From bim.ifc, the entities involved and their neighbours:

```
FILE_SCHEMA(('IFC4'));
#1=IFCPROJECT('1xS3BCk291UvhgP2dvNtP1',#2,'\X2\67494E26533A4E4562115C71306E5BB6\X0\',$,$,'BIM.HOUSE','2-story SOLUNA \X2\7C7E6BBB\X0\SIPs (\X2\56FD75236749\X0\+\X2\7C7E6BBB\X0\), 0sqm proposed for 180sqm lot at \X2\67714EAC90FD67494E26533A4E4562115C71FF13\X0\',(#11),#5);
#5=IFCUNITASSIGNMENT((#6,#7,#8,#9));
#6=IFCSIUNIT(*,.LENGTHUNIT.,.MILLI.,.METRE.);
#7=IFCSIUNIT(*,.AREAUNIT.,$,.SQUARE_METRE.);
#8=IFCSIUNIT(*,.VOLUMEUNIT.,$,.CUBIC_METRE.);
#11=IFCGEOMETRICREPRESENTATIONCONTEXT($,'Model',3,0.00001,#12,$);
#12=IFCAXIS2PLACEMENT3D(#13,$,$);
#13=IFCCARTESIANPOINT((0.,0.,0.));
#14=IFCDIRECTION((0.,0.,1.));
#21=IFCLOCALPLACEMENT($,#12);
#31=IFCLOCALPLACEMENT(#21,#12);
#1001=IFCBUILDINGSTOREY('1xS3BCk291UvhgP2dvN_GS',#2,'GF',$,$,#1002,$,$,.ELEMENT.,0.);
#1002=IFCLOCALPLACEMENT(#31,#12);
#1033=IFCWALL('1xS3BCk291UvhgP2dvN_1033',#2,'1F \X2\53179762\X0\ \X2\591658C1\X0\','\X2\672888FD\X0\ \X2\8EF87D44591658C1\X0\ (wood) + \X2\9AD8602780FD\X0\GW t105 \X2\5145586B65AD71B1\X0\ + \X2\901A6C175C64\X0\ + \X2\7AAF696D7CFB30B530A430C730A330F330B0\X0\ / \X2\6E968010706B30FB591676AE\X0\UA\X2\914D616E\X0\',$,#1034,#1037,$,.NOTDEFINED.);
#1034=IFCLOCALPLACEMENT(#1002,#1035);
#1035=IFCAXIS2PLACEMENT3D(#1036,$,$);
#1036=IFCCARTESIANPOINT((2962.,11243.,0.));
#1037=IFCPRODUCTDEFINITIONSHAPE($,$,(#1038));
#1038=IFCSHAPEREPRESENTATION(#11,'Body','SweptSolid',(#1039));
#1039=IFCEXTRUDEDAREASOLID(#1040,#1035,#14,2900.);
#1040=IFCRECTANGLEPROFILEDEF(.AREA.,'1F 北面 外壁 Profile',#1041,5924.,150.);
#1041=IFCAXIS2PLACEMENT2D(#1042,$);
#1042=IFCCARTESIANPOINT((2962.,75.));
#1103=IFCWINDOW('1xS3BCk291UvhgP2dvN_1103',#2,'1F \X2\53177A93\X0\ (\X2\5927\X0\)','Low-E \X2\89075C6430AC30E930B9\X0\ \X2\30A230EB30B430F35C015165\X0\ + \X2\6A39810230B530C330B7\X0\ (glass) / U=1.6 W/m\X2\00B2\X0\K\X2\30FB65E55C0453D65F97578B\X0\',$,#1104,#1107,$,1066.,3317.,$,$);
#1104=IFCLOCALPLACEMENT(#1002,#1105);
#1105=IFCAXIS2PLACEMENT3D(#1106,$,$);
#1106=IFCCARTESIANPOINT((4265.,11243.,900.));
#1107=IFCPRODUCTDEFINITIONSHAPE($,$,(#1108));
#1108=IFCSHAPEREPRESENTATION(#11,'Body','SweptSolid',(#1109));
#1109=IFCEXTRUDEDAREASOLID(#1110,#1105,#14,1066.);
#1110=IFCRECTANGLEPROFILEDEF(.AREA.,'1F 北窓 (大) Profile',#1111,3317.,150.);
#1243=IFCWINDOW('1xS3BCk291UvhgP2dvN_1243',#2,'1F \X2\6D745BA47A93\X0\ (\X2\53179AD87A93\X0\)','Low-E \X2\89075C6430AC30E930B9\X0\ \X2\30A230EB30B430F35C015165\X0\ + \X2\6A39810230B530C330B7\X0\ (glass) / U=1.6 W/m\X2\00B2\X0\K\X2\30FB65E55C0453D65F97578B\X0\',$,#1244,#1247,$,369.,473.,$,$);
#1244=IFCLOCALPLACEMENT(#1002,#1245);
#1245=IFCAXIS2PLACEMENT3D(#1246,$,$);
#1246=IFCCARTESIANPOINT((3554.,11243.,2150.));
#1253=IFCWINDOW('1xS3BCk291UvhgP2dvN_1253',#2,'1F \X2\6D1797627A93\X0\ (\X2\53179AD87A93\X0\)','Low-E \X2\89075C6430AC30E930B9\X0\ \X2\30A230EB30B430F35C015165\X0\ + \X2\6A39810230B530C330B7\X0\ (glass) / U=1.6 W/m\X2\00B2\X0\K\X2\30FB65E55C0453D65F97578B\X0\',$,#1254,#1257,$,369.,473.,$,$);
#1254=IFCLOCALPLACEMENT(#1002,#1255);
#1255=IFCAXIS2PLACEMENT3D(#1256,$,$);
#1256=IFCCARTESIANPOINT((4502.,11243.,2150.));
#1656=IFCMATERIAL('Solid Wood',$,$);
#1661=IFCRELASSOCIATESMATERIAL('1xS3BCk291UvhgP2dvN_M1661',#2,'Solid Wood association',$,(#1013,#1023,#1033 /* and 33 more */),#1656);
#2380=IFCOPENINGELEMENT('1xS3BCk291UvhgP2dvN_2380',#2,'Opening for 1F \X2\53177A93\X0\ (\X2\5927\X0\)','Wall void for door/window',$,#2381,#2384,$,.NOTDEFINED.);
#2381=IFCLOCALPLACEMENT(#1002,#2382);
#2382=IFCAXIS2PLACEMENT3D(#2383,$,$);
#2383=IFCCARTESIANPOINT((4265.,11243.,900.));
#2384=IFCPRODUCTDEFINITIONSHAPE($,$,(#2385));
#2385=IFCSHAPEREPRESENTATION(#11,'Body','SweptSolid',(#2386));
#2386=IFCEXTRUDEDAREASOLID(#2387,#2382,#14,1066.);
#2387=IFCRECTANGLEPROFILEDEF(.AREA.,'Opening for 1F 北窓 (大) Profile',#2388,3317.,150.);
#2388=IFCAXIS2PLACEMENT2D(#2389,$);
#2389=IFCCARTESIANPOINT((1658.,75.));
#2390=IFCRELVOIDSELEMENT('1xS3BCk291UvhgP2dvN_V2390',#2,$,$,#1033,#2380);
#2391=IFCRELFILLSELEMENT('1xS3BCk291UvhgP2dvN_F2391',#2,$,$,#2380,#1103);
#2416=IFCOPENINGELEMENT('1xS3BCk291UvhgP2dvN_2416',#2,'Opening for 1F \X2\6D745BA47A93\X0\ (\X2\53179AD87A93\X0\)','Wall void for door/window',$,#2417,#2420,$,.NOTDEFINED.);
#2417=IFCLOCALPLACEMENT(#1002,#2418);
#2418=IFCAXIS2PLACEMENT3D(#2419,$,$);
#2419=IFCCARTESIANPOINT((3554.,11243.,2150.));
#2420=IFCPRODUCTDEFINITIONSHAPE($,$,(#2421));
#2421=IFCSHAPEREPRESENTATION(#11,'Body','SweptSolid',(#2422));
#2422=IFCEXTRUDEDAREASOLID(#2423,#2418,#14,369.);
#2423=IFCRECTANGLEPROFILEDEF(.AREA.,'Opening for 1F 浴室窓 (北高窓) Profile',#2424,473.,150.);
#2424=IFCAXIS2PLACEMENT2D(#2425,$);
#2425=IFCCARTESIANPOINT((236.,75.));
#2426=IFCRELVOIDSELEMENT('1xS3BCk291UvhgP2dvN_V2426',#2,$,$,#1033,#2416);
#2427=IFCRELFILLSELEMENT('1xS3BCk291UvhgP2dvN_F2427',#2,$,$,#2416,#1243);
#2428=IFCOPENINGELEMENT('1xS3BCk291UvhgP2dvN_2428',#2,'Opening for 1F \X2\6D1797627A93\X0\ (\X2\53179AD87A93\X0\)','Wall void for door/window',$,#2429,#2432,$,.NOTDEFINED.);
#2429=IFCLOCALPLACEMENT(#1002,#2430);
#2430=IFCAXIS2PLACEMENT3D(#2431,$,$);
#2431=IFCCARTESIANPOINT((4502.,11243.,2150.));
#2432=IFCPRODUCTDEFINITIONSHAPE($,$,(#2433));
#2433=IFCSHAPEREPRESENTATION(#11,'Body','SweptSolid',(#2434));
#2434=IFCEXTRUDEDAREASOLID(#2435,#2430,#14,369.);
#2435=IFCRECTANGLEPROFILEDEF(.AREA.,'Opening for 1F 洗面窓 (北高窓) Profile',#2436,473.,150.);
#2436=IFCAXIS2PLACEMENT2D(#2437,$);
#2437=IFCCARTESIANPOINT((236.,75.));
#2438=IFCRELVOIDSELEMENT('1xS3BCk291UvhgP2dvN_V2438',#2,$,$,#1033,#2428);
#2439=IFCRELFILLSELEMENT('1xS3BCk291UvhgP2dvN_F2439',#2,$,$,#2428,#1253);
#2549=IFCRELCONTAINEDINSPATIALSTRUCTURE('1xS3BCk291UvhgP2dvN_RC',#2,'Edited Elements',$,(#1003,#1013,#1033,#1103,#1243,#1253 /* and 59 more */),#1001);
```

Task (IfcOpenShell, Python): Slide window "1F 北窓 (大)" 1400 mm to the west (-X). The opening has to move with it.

```python
import ifcopenshell
import ifcopenshell.api.geometry
import ifcopenshell.util.placement
import ifcopenshell.util.unit

model = ifcopenshell.open("bim.ifc")
unit_scale = ifcopenshell.util.unit.calculate_unit_scale(model)

window = model.by_guid("1xS3BCk291UvhgP2dvN_1103")
opening = window.FillsVoids[0].RelatingOpeningElement
wall = opening.VoidsElements[0].RelatingBuildingElement

wall_matrix = ifcopenshell.util.placement.get_local_placement(wall.ObjectPlacement)
shift = wall_matrix[:3, 0] * -1.4 / unit_scale
before = ifcopenshell.util.placement.get_local_placement(window.ObjectPlacement)[:3, 3].copy()

# The window is not placed relative to its opening, so move both.
for product in (opening, window):
    matrix = ifcopenshell.util.placement.get_local_placement(product.ObjectPlacement)
    matrix[:3, 3] += shift
    ifcopenshell.api.geometry.edit_object_placement(model, product=product, matrix=matrix, is_si=False)

after = ifcopenshell.util.placement.get_local_placement(window.ObjectPlacement)[:3, 3]
print("window moved by", (after - before).round(3) + 0.0)

model.write("bim_v2.ifc")
```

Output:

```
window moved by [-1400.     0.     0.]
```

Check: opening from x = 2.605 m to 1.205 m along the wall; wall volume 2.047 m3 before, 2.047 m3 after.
